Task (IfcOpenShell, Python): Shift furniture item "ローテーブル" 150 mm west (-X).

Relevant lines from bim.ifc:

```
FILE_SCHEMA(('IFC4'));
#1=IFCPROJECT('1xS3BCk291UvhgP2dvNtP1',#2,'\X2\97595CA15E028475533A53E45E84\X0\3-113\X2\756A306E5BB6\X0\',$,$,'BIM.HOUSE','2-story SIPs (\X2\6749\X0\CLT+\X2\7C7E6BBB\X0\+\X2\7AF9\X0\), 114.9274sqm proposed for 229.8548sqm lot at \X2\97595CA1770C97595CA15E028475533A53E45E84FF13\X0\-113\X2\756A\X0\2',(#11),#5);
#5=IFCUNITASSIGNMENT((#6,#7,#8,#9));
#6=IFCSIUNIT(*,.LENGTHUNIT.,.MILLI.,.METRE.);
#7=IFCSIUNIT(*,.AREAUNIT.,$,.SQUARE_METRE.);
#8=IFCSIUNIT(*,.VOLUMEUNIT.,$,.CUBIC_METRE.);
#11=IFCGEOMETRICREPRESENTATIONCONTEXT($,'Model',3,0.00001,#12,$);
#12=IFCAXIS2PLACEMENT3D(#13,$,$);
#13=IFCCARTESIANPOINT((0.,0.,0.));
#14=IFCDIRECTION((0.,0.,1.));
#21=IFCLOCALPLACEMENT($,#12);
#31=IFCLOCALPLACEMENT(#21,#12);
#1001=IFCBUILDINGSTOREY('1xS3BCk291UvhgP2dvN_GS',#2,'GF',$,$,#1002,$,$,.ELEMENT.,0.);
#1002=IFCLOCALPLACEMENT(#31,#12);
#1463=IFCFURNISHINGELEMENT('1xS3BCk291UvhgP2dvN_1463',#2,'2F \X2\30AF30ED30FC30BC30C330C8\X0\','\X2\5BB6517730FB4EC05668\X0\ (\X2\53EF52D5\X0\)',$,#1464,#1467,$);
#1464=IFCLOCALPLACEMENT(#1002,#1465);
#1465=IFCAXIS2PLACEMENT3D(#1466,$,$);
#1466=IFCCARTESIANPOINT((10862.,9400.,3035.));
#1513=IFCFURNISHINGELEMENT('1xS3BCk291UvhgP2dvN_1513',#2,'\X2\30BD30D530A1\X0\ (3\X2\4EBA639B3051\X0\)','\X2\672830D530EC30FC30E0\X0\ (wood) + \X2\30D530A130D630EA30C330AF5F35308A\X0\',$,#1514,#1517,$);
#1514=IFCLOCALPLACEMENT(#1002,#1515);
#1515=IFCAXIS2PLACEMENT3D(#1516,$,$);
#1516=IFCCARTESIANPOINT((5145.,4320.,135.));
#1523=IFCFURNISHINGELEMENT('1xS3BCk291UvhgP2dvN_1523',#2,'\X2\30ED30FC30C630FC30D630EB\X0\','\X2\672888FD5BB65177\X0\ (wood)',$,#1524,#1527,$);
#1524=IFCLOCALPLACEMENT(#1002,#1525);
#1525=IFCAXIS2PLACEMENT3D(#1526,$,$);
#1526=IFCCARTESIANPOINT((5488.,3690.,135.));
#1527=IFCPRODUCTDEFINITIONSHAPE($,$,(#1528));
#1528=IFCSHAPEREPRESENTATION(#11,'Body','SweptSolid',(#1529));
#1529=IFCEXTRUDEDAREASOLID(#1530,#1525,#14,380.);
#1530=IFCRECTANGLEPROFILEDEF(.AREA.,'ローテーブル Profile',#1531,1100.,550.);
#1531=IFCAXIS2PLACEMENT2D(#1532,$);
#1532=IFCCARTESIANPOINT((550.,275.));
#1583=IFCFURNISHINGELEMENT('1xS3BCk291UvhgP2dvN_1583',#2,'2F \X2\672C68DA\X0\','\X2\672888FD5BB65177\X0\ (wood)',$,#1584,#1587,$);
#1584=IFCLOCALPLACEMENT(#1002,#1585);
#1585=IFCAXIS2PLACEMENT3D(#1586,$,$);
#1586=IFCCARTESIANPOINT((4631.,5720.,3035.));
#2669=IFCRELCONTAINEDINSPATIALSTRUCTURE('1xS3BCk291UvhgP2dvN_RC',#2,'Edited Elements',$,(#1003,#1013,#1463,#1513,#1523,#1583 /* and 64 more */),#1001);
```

```python
import ifcopenshell
import ifcopenshell.api.geometry
import ifcopenshell.util.placement

model = ifcopenshell.open("bim.ifc")

item = model.by_guid("1xS3BCk291UvhgP2dvN_1523")
matrix = ifcopenshell.util.placement.get_local_placement(item.ObjectPlacement)
matrix[0, 3] -= 150.0
ifcopenshell.api.geometry.edit_object_placement(model, product=item, matrix=matrix, is_si=False)

print(ifcopenshell.util.placement.get_local_placement(item.ObjectPlacement).round(3) + 0.0)

model.write("bim-out.ifc")
```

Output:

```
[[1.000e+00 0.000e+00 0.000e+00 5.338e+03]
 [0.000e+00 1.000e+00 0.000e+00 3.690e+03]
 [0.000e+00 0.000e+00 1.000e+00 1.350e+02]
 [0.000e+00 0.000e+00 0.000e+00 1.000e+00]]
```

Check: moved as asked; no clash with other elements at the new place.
